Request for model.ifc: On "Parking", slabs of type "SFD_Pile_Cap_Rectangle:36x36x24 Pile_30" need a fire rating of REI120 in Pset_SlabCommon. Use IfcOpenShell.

First a look at what the model holds.

```python
import ifcopenshell
import ifcopenshell.util.element

model = ifcopenshell.open("model.ifc")
print(model.schema)
storey = next(s for s in model.by_type("IfcBuildingStorey") if s.Name == "Parking")
slabs = [e for e in ifcopenshell.util.element.get_decomposition(storey) if e.is_a("IfcSlab")]
seen = {}
for e in slabs:
    element_type = ifcopenshell.util.element.get_type(e)
    key = (element_type.Name if element_type != e and element_type else None, ifcopenshell.util.element.get_pset(e, "Pset_SlabCommon", "FireRating"))
    seen[key] = seen.get(key, 0) + 1
for (name, value), count in sorted(seen.items(), key=str):
    print(count, "x", name, "|", value)
```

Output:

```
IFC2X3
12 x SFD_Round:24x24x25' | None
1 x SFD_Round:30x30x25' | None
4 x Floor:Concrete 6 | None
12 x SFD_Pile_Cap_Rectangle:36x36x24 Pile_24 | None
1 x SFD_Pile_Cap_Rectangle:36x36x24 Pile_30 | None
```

```python
import ifcopenshell
import ifcopenshell.api.pset
import ifcopenshell.util.element

model = ifcopenshell.open("model.ifc")

storey = next(s for s in model.by_type("IfcBuildingStorey") if s.Name == "Parking")
slabs = [e for e in ifcopenshell.util.element.get_decomposition(storey) if e.is_a("IfcSlab")]

count = 0
for e in slabs:
    element_type = ifcopenshell.util.element.get_type(e)
    if element_type in (None, e) or element_type.Name != "SFD_Pile_Cap_Rectangle:36x36x24 Pile_30":
        continue
    # add_pset returns the element's existing set when there is one.
    pset = ifcopenshell.api.pset.add_pset(model, product=e, name="Pset_SlabCommon")
    ifcopenshell.api.pset.edit_pset(model, pset=pset, properties={"FireRating": "REI120"})
    count += 1

print(count, "slabs updated")

model.write("model_edited.ifc")
```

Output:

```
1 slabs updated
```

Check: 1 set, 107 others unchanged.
